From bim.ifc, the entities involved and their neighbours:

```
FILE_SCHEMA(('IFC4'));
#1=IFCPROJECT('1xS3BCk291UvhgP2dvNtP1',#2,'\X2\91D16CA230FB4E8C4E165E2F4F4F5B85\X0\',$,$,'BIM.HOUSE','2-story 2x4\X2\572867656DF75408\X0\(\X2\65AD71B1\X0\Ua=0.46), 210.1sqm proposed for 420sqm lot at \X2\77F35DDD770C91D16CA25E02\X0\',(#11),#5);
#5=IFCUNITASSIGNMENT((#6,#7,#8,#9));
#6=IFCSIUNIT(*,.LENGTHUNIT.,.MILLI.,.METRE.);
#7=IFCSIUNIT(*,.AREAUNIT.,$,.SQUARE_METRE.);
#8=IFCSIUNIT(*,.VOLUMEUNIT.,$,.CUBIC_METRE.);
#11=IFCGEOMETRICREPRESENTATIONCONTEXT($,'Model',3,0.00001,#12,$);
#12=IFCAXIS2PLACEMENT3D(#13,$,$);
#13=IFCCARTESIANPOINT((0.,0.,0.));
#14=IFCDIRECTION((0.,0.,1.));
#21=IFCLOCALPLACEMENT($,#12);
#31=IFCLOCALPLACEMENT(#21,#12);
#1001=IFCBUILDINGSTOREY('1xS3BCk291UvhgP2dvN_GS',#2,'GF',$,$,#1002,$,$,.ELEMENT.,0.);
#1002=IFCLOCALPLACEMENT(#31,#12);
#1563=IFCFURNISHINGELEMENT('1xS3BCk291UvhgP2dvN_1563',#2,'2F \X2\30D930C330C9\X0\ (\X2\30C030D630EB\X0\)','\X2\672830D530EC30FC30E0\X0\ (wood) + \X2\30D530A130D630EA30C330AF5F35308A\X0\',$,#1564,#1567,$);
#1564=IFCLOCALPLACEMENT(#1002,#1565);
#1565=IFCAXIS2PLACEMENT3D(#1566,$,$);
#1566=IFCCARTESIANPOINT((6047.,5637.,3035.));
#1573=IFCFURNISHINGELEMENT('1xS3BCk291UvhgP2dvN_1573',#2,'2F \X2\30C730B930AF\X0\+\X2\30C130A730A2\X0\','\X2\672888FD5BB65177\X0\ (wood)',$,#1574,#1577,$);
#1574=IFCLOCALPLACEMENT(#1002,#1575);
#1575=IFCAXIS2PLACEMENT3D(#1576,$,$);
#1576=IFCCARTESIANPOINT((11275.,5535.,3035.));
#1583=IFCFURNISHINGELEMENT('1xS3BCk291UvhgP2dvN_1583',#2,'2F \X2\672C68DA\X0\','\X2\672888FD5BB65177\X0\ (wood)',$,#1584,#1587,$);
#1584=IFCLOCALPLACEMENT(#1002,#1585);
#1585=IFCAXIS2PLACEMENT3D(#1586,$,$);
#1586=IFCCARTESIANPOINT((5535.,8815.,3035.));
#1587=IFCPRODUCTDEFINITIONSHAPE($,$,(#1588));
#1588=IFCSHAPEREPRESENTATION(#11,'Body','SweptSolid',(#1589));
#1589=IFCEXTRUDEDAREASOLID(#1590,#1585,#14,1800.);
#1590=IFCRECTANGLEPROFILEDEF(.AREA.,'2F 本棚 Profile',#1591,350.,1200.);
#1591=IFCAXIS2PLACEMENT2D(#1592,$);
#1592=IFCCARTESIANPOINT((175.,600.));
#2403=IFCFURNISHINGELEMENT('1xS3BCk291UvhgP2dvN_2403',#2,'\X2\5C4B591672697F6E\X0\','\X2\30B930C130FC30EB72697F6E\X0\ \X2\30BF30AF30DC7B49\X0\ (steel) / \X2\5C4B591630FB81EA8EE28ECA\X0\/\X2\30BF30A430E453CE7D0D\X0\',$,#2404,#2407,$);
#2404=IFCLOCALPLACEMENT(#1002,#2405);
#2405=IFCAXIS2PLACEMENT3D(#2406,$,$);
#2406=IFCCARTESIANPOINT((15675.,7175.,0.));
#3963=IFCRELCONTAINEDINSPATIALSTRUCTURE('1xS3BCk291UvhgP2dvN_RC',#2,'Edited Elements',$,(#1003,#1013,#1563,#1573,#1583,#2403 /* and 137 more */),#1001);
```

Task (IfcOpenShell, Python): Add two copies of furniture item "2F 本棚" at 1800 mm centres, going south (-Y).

```python
import numpy as np
import ifcopenshell
import ifcopenshell.api.geometry
import ifcopenshell.api.root
import ifcopenshell.util.element
import ifcopenshell.util.placement
import ifcopenshell.util.unit

model = ifcopenshell.open("bim.ifc")
unit_scale = ifcopenshell.util.unit.calculate_unit_scale(model)


def reuse_history(source, copy):
    """copy_class also copies each property set's owner history, people and application; keep the originals."""
    for rel in copy.IsDefinedBy:
        if rel.is_a("IfcRelDefinesByProperties") and (history := rel.RelatingPropertyDefinition.OwnerHistory):
            rel.RelatingPropertyDefinition.OwnerHistory = source.OwnerHistory
            ifcopenshell.util.element.remove_deep2(model, history)


source = model.by_guid("1xS3BCk291UvhgP2dvN_1583")
base = ifcopenshell.util.placement.get_local_placement(source.ObjectPlacement)
step = np.array([0.0, -1.0, 0.0]) * 1.8 / unit_scale

for i in range(1, 3):
    copy = ifcopenshell.api.root.copy_class(model, product=source)
    copy.Representation = ifcopenshell.util.element.copy_deep(
        model, source.Representation, exclude=["IfcGeometricRepresentationContext", "IfcRepresentationMap"]
    )
    reuse_history(source, copy)
    matrix = base.copy()
    matrix[:3, 3] += i * step
    print("added at", matrix[:3, 3].round(3) + 0.0)
    ifcopenshell.api.geometry.edit_object_placement(model, product=copy, matrix=matrix, is_si=False)

model.write("bim_updated.ifc")
```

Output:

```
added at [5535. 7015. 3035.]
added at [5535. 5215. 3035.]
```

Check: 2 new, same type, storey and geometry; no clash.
